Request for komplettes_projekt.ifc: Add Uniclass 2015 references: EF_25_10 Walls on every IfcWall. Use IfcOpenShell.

First a look at what the model holds.

```python
import ifcopenshell

model = ifcopenshell.open("komplettes_projekt.ifc")
print(model.schema)
print("classifications:", [c.Name for c in model.by_type("IfcClassification")])
for ifc_class in ("IfcDoor", "IfcRoof", "IfcStair", "IfcWall", "IfcWindow"):
    print(ifc_class, len(model.by_type(ifc_class)))
```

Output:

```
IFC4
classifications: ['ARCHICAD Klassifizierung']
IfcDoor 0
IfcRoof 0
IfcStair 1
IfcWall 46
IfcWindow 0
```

```python
import ifcopenshell
import ifcopenshell.api.classification

model = ifcopenshell.open("komplettes_projekt.ifc")

system = ifcopenshell.api.classification.add_classification(model, classification="Uniclass 2015")

codes = {
    "IfcWall": ("EF_25_10", "Walls"),
}
for ifc_class, (code, name) in codes.items():
    products = model.by_type(ifc_class)
    ifcopenshell.api.classification.add_reference(
        model, products=products, classification=system, identification=code, name=name
    )
    print(code, len(products))

model.write("komplettes_projekt_edited.ifc")
```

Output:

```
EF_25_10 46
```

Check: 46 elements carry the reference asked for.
